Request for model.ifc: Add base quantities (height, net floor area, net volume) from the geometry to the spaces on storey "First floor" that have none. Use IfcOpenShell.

First a look at what the model holds.

```python
import ifcopenshell
import ifcopenshell.util.element
import ifcopenshell.util.unit

model = ifcopenshell.open("model.ifc")
print(model.schema)
for unit_type in ("LENGTHUNIT", "AREAUNIT", "VOLUMEUNIT"):
    print(unit_type, ifcopenshell.util.unit.calculate_unit_scale(model, unit_type))
storey = next(s for s in model.by_type("IfcBuildingStorey") if s.Name == "First floor")
spaces = [e for e in ifcopenshell.util.element.get_decomposition(storey) if e.is_a("IfcSpace")]
for e in sorted(spaces, key=lambda e: e.id()):
    print(e.id(), e.is_a(), e.Name, list(ifcopenshell.util.element.get_psets(e, qtos_only=True)), sep=" | ")
```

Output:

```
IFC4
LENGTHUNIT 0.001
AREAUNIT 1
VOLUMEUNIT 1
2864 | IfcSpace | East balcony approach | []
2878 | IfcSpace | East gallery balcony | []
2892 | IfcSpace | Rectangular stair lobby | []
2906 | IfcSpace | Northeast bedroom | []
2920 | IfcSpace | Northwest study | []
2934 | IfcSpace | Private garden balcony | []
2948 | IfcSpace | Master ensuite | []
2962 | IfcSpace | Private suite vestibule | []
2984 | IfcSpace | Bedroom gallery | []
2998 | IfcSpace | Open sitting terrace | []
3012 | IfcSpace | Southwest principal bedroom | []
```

```python
import ifcopenshell
import ifcopenshell.api.pset
import ifcopenshell.geom
import ifcopenshell.util.element
import ifcopenshell.util.shape
import ifcopenshell.util.unit

model = ifcopenshell.open("model.ifc")
unit_scale = ifcopenshell.util.unit.calculate_unit_scale(model)
area_scale = ifcopenshell.util.unit.calculate_unit_scale(model, "AREAUNIT")
volume_scale = ifcopenshell.util.unit.calculate_unit_scale(model, "VOLUMEUNIT")
settings = ifcopenshell.geom.settings()

storey = next(s for s in model.by_type("IfcBuildingStorey") if s.Name == "First floor")
spaces = [e for e in ifcopenshell.util.element.get_decomposition(storey) if e.is_a("IfcSpace")]

for e in sorted(spaces, key=lambda e: e.id()):
    if ifcopenshell.util.element.get_psets(e, qtos_only=True, should_inherit=False):
        continue
    # Geometry comes back in metres, in the element's own axes.
    shape = ifcopenshell.geom.create_shape(settings, e)
    values = {
        "Height": ifcopenshell.util.shape.get_z(shape.geometry) / unit_scale,
        "NetFloorArea": ifcopenshell.util.shape.get_footprint_area(shape.geometry) / area_scale,
        "NetVolume": ifcopenshell.util.shape.get_volume(shape.geometry) / volume_scale,
    }
    qto = ifcopenshell.api.pset.add_qto(model, product=e, name="Qto_SpaceBaseQuantities")
    ifcopenshell.api.pset.edit_qto(model, qto=qto, properties=values)
    print(e.id(), {k: round(v, 3) for k, v in values.items()})

model.write("model_v2.ifc")
```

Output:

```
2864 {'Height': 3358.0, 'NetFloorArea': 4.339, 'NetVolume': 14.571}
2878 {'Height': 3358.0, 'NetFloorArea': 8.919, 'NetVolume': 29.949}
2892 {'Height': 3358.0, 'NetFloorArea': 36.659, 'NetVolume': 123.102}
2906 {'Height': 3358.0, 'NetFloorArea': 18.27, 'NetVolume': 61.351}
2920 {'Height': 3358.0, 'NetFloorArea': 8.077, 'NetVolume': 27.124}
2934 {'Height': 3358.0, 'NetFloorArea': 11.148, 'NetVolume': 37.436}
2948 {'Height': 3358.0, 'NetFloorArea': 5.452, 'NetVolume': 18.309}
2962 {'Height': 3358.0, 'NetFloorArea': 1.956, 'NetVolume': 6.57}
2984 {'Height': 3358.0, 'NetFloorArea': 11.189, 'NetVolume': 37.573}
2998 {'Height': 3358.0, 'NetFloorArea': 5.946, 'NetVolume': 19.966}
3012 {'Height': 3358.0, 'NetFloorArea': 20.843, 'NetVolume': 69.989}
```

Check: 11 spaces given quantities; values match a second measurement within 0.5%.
